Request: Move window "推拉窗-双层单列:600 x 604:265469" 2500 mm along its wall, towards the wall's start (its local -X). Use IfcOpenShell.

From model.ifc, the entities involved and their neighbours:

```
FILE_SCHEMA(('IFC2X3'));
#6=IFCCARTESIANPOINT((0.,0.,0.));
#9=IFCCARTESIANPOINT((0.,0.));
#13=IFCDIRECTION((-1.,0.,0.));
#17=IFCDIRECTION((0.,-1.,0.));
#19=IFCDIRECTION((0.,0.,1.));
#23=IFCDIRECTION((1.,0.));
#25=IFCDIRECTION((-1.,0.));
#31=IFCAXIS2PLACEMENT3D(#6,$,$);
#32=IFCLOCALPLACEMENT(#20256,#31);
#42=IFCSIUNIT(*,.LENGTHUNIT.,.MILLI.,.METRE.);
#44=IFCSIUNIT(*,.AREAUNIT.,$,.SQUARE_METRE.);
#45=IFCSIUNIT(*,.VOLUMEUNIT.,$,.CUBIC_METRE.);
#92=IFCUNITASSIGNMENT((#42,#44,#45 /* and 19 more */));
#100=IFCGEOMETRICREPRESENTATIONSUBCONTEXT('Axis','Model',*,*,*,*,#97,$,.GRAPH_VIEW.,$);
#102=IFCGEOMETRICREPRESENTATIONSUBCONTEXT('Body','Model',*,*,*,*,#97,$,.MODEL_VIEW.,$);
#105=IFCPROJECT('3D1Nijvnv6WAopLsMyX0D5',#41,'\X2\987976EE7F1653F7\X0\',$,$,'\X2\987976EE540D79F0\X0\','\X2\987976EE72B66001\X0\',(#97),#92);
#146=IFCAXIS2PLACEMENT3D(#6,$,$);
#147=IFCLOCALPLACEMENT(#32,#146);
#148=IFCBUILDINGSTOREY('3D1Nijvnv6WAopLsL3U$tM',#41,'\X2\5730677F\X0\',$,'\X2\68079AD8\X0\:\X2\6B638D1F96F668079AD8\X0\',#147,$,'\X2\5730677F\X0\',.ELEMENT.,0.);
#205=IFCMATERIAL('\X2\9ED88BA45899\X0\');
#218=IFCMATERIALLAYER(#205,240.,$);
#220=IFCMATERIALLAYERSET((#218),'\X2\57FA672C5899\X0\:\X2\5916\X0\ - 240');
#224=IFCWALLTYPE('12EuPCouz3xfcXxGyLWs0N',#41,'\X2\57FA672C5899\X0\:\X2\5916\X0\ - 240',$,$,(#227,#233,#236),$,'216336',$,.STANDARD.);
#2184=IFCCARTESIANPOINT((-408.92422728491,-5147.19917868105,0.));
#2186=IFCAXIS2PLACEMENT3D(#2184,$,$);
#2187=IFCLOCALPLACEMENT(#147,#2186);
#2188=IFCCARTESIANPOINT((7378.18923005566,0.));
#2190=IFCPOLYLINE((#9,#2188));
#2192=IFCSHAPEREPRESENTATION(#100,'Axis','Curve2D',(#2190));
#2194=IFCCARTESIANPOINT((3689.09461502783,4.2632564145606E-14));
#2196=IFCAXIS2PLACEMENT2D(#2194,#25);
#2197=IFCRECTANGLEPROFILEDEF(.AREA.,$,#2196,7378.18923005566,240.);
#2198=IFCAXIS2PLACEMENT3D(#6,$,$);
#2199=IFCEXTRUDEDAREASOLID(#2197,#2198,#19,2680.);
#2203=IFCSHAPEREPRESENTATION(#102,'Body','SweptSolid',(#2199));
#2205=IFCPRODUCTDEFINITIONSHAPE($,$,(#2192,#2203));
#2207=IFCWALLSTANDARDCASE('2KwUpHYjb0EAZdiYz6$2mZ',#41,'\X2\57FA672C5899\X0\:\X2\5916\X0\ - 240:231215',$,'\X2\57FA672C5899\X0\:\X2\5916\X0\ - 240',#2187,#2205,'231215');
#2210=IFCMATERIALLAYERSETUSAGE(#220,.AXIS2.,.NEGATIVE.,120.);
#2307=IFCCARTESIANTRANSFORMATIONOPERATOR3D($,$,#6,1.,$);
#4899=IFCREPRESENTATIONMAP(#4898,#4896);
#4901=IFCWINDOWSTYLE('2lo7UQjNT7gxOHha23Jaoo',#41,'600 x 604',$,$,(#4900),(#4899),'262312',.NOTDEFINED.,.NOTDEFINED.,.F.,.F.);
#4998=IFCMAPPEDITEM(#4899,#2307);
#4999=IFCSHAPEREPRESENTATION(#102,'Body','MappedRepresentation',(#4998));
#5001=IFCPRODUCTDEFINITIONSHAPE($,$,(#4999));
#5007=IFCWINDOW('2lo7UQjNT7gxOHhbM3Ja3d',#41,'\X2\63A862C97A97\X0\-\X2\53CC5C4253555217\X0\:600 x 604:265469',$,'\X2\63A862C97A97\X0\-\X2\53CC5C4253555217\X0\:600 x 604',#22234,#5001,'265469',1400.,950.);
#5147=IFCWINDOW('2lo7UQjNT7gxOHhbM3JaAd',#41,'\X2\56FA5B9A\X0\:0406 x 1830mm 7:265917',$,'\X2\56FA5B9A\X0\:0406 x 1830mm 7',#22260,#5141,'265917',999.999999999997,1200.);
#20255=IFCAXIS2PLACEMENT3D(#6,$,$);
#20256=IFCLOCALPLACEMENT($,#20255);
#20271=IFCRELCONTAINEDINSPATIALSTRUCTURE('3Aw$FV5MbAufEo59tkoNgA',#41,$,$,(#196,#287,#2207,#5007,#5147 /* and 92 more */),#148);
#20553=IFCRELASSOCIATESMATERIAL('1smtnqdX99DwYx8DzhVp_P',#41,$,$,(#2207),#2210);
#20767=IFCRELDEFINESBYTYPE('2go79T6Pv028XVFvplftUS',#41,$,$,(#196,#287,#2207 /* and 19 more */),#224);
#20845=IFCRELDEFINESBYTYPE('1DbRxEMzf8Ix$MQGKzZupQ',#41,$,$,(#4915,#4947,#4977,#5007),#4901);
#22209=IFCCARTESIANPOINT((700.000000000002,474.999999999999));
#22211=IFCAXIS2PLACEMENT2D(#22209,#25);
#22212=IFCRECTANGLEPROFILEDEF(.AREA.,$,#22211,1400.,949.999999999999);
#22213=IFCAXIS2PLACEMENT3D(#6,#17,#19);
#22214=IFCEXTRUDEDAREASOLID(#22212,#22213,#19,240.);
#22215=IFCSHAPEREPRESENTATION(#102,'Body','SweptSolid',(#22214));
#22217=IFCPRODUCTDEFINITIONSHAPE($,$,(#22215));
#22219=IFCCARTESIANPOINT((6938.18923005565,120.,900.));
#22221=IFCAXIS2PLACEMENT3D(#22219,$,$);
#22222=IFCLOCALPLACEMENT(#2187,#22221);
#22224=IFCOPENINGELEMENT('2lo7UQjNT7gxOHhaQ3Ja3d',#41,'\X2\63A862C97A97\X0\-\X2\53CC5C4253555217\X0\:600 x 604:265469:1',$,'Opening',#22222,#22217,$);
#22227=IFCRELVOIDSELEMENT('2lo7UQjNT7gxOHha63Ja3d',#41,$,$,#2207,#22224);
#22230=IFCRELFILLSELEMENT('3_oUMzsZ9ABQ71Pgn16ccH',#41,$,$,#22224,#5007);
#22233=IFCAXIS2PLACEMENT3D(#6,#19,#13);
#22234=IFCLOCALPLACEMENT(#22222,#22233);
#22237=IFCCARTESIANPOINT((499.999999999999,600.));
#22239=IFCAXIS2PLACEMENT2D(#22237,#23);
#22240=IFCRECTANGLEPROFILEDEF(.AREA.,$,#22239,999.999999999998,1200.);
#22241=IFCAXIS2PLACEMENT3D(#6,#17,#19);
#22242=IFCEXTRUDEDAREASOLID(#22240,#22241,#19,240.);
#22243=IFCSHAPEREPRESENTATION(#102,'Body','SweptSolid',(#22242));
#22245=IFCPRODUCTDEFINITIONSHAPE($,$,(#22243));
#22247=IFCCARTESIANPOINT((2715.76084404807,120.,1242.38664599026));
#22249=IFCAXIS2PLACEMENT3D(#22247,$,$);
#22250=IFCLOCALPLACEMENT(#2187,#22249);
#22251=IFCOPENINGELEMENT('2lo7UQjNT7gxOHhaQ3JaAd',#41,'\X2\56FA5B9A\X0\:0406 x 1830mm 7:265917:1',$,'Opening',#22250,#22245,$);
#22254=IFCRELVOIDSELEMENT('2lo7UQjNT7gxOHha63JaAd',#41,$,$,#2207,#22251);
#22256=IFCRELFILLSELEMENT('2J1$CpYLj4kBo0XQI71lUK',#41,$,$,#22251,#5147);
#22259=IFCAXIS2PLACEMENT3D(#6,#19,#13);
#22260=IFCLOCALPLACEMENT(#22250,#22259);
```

```python
import ifcopenshell
import ifcopenshell.api.geometry
import ifcopenshell.util.placement

model = ifcopenshell.open("model.ifc")

window = model.by_guid("2lo7UQjNT7gxOHhbM3Ja3d")
opening = window.FillsVoids[0].RelatingOpeningElement
wall = opening.VoidsElements[0].RelatingBuildingElement

wall_matrix = ifcopenshell.util.placement.get_local_placement(wall.ObjectPlacement)
shift = wall_matrix[:3, 0] * -2500.0
before = ifcopenshell.util.placement.get_local_placement(window.ObjectPlacement)[:3, 3].copy()

# The window is placed relative to its opening, so it follows when the opening moves.
matrix = ifcopenshell.util.placement.get_local_placement(opening.ObjectPlacement)
matrix[:3, 3] += shift
ifcopenshell.api.geometry.edit_object_placement(
    model, product=opening, matrix=matrix, is_si=False, should_transform_children=True
)

after = ifcopenshell.util.placement.get_local_placement(window.ObjectPlacement)[:3, 3]
print("window moved by", (after - before).round(3) + 0.0)

model.write("model-out.ifc")
```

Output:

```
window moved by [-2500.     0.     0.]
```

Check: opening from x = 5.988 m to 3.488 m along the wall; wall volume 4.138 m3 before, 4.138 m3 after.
